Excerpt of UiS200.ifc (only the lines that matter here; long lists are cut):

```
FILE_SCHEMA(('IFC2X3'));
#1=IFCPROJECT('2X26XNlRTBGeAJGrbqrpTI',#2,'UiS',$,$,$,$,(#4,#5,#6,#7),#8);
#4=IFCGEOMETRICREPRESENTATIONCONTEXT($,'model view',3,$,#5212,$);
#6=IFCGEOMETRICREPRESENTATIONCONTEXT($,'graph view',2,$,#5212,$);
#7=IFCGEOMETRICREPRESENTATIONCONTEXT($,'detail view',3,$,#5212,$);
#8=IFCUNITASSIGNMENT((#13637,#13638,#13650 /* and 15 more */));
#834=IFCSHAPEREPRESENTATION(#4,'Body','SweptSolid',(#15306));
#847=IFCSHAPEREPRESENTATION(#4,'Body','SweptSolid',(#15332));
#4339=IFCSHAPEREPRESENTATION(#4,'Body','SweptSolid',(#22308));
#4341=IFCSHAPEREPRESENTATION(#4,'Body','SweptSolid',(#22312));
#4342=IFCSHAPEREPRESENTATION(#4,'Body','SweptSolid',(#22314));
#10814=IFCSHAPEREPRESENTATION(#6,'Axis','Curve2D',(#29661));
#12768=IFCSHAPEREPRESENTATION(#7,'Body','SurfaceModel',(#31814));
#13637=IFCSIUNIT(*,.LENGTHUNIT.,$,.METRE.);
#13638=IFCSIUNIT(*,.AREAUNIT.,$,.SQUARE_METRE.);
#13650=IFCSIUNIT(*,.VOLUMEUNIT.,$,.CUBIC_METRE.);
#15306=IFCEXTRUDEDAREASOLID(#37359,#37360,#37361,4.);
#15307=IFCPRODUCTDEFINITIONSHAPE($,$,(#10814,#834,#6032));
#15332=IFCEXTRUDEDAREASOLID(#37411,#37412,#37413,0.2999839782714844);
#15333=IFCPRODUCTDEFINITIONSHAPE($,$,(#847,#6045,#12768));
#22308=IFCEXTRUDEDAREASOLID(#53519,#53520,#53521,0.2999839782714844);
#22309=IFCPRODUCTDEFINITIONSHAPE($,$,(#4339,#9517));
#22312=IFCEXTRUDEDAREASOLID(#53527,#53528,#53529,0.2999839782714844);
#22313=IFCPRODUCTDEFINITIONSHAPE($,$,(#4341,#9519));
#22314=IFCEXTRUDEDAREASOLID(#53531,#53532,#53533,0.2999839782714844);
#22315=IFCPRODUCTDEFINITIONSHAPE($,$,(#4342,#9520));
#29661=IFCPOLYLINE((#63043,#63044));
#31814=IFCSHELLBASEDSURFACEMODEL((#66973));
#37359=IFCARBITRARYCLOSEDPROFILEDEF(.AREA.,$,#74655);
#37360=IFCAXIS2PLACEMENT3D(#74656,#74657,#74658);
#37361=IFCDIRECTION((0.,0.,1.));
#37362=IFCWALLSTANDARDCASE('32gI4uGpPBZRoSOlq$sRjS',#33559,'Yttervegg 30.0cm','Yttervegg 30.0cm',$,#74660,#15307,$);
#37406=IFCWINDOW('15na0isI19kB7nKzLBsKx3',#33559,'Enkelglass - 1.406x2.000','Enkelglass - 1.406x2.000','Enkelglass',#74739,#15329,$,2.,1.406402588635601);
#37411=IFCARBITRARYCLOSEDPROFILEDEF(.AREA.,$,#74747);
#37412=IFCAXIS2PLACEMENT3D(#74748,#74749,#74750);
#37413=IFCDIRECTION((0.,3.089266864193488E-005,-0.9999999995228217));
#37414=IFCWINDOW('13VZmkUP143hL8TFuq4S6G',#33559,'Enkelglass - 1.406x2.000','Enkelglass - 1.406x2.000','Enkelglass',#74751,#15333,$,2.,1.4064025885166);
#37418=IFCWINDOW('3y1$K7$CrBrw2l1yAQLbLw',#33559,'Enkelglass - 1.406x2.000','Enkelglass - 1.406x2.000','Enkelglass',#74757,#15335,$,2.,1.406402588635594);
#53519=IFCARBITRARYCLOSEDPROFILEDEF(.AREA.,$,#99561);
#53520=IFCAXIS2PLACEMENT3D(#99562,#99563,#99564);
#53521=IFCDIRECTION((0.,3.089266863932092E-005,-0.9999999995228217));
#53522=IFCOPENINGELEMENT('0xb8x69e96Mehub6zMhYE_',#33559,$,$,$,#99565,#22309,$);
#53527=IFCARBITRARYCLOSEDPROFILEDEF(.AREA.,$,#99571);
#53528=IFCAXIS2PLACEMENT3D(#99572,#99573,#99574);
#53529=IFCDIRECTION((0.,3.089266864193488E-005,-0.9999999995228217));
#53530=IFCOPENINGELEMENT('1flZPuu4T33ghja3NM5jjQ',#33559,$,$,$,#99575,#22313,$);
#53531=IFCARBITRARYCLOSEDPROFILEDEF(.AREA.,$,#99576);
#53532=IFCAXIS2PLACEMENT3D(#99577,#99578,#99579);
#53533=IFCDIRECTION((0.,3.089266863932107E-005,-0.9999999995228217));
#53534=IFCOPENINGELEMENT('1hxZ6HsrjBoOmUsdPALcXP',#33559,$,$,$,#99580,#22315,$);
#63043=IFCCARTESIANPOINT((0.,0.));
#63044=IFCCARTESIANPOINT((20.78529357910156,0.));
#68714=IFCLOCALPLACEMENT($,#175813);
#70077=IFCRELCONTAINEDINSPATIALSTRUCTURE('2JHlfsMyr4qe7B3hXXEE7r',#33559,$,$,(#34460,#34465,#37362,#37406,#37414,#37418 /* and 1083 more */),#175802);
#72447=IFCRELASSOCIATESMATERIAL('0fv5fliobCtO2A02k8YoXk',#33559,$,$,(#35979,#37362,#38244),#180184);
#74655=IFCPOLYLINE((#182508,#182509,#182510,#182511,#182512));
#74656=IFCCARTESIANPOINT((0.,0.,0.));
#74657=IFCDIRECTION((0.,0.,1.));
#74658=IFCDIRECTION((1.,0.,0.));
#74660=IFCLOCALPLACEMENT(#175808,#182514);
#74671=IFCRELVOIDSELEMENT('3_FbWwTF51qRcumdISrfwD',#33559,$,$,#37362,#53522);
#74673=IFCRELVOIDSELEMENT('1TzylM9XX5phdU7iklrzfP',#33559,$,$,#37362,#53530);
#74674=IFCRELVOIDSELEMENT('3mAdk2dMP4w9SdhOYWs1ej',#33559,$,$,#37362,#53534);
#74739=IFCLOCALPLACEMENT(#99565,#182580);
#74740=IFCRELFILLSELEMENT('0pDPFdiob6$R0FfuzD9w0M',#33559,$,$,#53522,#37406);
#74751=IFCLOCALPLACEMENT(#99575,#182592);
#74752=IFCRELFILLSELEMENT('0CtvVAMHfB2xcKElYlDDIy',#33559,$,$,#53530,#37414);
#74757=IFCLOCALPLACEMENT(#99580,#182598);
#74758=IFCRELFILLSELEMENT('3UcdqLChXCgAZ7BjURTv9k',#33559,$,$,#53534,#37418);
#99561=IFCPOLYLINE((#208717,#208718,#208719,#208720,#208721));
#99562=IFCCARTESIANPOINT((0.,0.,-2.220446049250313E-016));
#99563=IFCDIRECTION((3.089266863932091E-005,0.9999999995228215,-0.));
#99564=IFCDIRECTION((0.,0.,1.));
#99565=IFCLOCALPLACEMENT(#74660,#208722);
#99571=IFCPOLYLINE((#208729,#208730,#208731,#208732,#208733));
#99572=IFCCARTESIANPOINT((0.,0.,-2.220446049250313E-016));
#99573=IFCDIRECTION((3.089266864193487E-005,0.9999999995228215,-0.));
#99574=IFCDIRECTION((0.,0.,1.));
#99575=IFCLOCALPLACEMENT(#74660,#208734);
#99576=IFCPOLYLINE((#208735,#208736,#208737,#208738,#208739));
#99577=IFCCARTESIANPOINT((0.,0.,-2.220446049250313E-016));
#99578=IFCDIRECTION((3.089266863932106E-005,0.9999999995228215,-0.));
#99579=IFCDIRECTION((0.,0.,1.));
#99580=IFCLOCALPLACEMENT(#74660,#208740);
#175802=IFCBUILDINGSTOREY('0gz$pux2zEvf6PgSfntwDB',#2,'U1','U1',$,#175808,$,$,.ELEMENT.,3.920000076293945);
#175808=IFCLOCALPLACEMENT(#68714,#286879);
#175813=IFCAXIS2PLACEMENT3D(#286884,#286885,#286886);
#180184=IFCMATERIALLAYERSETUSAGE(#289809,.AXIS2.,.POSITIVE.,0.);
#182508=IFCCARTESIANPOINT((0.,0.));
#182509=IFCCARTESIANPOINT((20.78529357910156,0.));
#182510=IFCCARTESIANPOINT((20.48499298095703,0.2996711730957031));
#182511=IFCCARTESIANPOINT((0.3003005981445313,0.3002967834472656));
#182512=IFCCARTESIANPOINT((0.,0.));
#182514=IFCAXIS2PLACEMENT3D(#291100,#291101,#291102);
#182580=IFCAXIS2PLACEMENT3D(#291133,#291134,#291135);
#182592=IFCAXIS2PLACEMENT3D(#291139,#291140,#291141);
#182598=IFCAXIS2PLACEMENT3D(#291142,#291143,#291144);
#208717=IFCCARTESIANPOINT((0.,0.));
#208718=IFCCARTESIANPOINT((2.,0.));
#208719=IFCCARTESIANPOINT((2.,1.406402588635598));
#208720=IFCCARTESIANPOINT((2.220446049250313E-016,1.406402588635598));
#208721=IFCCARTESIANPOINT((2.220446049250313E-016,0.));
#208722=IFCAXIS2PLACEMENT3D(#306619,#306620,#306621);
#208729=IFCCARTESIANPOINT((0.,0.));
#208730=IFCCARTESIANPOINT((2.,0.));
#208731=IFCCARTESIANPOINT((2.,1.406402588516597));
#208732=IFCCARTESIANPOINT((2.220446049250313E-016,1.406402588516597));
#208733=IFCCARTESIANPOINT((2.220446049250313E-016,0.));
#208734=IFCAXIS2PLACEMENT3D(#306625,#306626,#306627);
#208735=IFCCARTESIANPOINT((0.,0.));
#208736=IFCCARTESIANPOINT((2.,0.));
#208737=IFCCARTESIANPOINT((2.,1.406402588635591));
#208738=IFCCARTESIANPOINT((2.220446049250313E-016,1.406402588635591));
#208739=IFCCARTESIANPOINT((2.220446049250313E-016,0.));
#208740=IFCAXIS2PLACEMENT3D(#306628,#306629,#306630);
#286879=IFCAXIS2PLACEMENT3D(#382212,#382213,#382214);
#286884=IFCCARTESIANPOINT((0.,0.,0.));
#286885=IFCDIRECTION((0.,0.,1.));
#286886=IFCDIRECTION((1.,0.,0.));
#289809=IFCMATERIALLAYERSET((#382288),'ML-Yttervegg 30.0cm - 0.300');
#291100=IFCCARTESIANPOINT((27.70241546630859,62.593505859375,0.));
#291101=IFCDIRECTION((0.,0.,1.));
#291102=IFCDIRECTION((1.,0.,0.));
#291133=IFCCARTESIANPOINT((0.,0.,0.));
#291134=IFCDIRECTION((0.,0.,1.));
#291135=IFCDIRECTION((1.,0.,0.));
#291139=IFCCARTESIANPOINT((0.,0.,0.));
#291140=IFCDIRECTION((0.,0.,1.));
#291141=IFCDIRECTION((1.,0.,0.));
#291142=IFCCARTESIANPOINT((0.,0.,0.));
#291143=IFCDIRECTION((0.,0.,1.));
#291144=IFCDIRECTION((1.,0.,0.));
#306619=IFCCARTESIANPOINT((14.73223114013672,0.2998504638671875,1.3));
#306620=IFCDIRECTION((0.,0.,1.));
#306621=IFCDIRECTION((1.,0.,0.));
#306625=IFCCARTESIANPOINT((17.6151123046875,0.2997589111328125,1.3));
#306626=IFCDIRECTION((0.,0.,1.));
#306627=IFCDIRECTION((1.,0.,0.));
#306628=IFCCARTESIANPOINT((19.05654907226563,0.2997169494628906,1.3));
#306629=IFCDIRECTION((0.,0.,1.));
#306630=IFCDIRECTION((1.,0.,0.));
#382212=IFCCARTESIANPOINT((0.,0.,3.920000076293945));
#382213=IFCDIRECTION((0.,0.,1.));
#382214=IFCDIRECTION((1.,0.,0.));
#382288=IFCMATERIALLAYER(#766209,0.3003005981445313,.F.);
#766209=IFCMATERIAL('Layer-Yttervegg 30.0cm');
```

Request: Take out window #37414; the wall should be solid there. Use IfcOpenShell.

```python
import ifcopenshell
import ifcopenshell.api.feature
import ifcopenshell.api.root
import ifcopenshell.geom
import ifcopenshell.util.shape

model = ifcopenshell.open("UiS200.ifc")
settings = ifcopenshell.geom.settings()


def volume(element):
    """Net volume in cubic metres, openings subtracted."""
    shape = ifcopenshell.geom.create_shape(settings, element)
    return ifcopenshell.util.shape.get_volume(shape.geometry)


window = model.by_id(37414)
opening = window.FillsVoids[0].RelatingOpeningElement
wall = opening.VoidsElements[0].RelatingBuildingElement
before = volume(wall)

ifcopenshell.api.root.remove_product(model, product=window)
ifcopenshell.api.feature.remove_feature(model, feature=opening)

after = volume(wall)

print(f"wall volume {before:.3f} -> {after:.3f} m3")

model.write("UiS200_rev.ifc")
```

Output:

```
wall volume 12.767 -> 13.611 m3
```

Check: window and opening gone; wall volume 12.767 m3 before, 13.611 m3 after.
